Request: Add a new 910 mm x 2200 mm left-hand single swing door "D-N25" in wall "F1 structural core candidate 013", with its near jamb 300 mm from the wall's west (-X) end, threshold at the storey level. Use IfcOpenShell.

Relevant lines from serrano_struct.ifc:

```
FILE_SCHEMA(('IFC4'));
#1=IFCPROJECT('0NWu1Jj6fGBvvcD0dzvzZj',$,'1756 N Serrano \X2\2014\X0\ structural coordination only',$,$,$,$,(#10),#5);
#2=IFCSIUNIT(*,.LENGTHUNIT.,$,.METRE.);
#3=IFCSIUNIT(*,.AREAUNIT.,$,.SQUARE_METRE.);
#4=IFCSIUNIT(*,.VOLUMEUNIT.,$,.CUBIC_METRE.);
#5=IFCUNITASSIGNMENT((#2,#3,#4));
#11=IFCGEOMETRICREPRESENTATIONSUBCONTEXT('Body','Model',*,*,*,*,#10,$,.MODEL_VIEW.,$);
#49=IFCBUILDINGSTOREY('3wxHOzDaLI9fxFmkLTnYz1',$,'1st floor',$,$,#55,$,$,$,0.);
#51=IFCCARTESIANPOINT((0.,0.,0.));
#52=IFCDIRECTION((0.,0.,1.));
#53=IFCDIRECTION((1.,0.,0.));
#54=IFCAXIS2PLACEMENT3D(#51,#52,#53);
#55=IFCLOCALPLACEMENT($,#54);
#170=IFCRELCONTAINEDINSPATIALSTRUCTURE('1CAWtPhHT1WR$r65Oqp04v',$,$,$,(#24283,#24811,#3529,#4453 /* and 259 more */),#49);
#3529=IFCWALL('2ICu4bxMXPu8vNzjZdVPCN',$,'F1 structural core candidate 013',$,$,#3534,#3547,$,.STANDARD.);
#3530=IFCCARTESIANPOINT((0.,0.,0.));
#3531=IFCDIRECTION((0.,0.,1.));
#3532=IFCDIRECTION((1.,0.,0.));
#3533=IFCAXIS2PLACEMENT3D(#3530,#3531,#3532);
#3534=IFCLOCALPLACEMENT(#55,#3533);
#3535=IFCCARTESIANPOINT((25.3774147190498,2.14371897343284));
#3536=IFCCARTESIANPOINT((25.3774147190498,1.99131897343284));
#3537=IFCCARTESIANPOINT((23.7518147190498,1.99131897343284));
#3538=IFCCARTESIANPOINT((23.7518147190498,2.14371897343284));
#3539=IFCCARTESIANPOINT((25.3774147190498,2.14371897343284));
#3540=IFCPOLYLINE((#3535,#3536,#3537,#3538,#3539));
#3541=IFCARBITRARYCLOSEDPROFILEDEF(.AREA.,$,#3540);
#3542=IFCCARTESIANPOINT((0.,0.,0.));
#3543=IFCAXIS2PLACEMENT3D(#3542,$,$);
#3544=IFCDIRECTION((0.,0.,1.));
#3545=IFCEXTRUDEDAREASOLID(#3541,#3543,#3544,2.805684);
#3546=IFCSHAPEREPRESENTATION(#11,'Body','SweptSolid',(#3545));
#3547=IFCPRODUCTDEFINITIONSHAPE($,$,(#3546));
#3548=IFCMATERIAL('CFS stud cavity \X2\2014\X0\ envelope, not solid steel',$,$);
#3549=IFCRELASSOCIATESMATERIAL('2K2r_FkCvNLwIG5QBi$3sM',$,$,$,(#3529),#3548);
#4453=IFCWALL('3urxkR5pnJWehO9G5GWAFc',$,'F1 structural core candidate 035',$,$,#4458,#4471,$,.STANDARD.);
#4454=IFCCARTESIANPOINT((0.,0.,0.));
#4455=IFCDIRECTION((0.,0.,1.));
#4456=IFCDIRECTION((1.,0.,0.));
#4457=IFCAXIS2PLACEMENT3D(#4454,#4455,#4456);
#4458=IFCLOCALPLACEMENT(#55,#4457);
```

```python
import numpy as np
import ifcopenshell
import ifcopenshell.api.feature
import ifcopenshell.api.geometry
import ifcopenshell.api.root
import ifcopenshell.api.spatial
import ifcopenshell.geom
import ifcopenshell.util.element
import ifcopenshell.util.placement
import ifcopenshell.util.representation
import ifcopenshell.util.shape
import ifcopenshell.util.unit

model = ifcopenshell.open("serrano_struct.ifc")
unit_scale = ifcopenshell.util.unit.calculate_unit_scale(model)
settings = ifcopenshell.geom.settings()


def volume(element):
    """Net volume in cubic metres, openings subtracted."""
    shape = ifcopenshell.geom.create_shape(settings, element)
    return ifcopenshell.util.shape.get_volume(shape.geometry)


wall = model.by_guid("2ICu4bxMXPu8vNzjZdVPCN")
storey = ifcopenshell.util.element.get_container(wall, ifc_class="IfcBuildingStorey")
context = ifcopenshell.util.representation.get_context(model, "Model", "Body", "MODEL_VIEW")
before = volume(wall)

width, height, from_end, sill = 0.91, 2.2, 0.3, 0.0  # metres

# The wall runs along its own X axis, and the end named is its -X end.
wall_shape = ifcopenshell.geom.create_shape(settings, wall)
x, y, z = ifcopenshell.util.shape.get_vertices(wall_shape.geometry).T
start = x.min() + from_end
face, thickness = float(y.min()), float(y.max() - y.min())
wall_matrix = ifcopenshell.util.placement.get_local_placement(wall.ObjectPlacement)
level = ifcopenshell.util.placement.get_local_placement(storey.ObjectPlacement)[2, 3]


def in_wall(x, y):
    """Placement at x, y metres in the wall's axes, at sill height."""
    matrix = wall_matrix.copy()
    matrix[:, 3] = wall_matrix @ np.array([x / unit_scale, y / unit_scale, 0.0, 1.0])
    matrix[2, 3] = level + sill / unit_scale
    return matrix


# Opening: a box that overshoots both wall faces by 50 mm.
opening = ifcopenshell.api.root.create_entity(model, ifc_class="IfcOpeningElement", predefined_type="OPENING")
box = ifcopenshell.api.geometry.add_wall_representation(
    model, context=context, length=width, height=height, thickness=thickness + 0.1
)
ifcopenshell.api.geometry.assign_representation(model, product=opening, representation=box)
ifcopenshell.api.geometry.edit_object_placement(model, product=opening, matrix=in_wall(start, face - 0.05), is_si=False)
ifcopenshell.api.feature.add_feature(model, feature=opening, element=wall)

door = ifcopenshell.api.root.create_entity(model, ifc_class="IfcDoor", name="D-N25", predefined_type="DOOR")
door.OverallWidth, door.OverallHeight = width / unit_scale, height / unit_scale
door.OperationType = "SINGLE_SWING_LEFT"
body = ifcopenshell.api.geometry.add_door_representation(
    model,
    context=context,
    overall_width=door.OverallWidth,
    overall_height=door.OverallHeight,
    operation_type="SINGLE_SWING_LEFT",
    lining_properties={"LiningDepth": thickness / unit_scale, "ThresholdDepth": thickness / unit_scale},
)
ifcopenshell.api.geometry.assign_representation(model, product=door, representation=body)
ifcopenshell.api.spatial.assign_container(model, products=[door], relating_structure=storey)
ifcopenshell.api.feature.add_filling(model, opening=opening, element=door)

# The lining spans the wall, so the door starts at the wall face.
ifcopenshell.api.geometry.edit_object_placement(model, product=door, matrix=in_wall(start, face), is_si=False)

after = volume(wall)

print(f"wall volume {before:.3f} -> {after:.3f} m3")

model.write("serrano_struct_edited.ifc")
```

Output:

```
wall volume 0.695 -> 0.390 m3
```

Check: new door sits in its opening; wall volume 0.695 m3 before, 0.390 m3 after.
